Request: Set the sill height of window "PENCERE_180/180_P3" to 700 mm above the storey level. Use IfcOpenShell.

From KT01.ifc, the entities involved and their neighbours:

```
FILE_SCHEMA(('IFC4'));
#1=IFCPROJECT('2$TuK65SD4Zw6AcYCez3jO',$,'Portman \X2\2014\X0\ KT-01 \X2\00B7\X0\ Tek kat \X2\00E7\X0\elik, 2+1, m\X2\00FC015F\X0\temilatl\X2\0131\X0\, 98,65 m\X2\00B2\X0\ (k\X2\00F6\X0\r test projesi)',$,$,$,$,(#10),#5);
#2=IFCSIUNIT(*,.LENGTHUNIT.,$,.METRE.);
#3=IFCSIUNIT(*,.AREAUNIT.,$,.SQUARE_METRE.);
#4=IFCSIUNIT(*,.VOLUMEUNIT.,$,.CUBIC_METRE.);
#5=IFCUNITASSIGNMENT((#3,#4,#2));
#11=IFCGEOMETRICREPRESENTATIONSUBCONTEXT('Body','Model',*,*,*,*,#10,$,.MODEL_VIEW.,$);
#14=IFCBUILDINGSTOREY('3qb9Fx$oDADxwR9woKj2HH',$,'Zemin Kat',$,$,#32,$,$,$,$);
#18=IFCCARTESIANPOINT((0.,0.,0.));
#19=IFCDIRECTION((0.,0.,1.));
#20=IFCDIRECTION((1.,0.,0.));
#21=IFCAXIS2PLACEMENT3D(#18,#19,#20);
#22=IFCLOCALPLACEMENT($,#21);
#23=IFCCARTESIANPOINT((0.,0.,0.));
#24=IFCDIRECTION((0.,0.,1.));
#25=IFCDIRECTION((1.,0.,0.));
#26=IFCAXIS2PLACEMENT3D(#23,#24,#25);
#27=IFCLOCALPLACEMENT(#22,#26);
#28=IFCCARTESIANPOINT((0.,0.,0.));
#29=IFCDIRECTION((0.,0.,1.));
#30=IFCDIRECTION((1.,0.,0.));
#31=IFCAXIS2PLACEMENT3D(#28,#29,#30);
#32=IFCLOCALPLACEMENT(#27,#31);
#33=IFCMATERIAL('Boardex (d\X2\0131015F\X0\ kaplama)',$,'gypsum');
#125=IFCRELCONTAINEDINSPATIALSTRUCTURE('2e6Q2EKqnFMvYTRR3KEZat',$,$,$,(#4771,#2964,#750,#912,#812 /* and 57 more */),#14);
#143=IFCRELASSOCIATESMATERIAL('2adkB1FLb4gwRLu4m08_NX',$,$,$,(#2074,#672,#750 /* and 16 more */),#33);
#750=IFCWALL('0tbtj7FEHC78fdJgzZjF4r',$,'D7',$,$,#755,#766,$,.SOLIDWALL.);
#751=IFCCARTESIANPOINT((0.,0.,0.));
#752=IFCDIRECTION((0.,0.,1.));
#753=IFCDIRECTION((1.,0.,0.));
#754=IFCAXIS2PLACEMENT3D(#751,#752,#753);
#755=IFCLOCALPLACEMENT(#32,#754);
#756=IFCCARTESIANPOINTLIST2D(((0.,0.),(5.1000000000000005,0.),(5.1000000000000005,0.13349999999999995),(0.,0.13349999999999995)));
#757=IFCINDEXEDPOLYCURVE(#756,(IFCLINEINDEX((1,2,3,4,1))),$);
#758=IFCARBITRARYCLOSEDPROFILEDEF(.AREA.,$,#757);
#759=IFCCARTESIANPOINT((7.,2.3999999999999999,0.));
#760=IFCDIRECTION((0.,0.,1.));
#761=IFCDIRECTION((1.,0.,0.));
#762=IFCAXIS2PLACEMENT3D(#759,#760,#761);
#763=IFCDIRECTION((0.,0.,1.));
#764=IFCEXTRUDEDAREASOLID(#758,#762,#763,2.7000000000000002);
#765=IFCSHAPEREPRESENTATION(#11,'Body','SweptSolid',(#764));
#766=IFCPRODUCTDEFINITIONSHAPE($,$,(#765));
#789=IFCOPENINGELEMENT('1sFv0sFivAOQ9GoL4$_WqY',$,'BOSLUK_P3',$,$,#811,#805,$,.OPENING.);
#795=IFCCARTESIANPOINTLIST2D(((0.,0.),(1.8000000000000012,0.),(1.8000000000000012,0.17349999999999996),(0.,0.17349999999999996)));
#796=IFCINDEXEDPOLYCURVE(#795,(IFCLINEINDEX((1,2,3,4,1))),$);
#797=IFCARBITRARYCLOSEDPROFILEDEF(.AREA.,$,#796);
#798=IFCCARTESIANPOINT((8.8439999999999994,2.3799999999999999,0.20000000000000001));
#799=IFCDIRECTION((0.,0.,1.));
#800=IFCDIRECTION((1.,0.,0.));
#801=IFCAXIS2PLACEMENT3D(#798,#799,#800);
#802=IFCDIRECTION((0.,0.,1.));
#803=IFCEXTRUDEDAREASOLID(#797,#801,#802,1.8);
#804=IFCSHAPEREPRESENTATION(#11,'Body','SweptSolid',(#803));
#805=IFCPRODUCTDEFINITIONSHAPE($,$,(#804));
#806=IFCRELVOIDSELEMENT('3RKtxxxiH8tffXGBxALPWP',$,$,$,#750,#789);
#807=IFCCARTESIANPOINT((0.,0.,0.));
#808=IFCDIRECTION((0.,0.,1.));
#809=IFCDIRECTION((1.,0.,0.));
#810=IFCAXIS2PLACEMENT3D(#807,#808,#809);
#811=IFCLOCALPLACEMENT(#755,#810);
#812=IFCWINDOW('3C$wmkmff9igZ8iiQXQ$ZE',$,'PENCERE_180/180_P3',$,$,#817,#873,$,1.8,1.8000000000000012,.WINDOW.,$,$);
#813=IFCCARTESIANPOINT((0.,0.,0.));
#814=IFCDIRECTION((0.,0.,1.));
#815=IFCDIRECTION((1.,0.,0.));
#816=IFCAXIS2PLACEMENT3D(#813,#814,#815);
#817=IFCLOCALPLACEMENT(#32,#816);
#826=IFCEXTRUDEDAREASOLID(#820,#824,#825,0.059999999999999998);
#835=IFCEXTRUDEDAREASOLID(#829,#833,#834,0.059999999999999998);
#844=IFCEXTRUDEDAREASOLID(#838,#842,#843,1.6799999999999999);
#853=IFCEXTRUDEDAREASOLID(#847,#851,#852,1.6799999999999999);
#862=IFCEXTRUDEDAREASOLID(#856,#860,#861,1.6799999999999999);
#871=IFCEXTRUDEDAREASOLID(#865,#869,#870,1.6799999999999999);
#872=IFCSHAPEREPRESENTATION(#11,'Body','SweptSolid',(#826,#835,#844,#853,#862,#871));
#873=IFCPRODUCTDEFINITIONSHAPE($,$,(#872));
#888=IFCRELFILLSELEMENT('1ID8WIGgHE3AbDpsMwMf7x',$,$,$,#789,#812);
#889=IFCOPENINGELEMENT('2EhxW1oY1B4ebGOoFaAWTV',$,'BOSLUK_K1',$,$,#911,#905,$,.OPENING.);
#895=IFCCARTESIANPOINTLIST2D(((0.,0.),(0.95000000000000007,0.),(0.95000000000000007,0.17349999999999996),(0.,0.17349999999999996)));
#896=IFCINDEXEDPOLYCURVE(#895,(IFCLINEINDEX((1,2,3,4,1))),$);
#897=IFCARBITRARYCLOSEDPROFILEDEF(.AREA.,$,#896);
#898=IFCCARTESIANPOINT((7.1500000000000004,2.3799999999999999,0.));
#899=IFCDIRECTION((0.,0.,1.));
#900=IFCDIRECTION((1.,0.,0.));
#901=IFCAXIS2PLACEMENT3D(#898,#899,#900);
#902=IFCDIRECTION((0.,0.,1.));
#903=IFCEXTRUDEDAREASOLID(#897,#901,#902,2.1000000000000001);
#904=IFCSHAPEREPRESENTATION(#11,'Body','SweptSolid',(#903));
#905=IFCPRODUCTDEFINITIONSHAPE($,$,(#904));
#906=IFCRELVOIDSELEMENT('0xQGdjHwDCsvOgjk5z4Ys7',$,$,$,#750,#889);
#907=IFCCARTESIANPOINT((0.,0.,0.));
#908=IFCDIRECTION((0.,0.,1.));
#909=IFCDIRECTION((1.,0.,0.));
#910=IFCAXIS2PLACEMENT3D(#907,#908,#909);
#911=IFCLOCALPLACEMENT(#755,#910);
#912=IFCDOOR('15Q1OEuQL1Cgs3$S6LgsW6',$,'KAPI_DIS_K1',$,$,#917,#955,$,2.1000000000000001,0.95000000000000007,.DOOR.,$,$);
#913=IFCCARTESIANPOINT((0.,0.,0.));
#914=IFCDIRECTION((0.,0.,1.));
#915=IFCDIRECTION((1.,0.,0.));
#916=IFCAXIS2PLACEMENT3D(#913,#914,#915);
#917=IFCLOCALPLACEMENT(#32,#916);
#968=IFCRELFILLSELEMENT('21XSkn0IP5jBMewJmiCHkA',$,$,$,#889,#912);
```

```python
import numpy as np
import ifcopenshell
import ifcopenshell.api.geometry
import ifcopenshell.geom
import ifcopenshell.util.element
import ifcopenshell.util.placement
import ifcopenshell.util.shape
import ifcopenshell.util.unit

model = ifcopenshell.open("KT01.ifc")
unit_scale = ifcopenshell.util.unit.calculate_unit_scale(model)

window = model.by_id(812)
opening = window.FillsVoids[0].RelatingOpeningElement
storey = ifcopenshell.util.element.get_container(window, ifc_class="IfcBuildingStorey")
level = ifcopenshell.util.placement.get_local_placement(storey.ObjectPlacement)[2, 3]

# The opening's origin need not be at the sill, so measure its lowest point.
shape = ifcopenshell.geom.create_shape(ifcopenshell.geom.settings(), opening)
bottom = ifcopenshell.util.shape.get_shape_bottom_elevation(shape, shape.geometry) / unit_scale
dz = level + 0.7 / unit_scale - bottom

shift = np.array([0.0, 0.0, dz])
# The window is not placed relative to its opening, so move both.
for product in (opening, window):
    matrix = ifcopenshell.util.placement.get_local_placement(product.ObjectPlacement)
    matrix[:3, 3] += shift
    ifcopenshell.api.geometry.edit_object_placement(model, product=product, matrix=matrix, is_si=False)

print(f"moved by {dz * unit_scale:+.3f} m")

model.write("KT01_rev.ifc")
```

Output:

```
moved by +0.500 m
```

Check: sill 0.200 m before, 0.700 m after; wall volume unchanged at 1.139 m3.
